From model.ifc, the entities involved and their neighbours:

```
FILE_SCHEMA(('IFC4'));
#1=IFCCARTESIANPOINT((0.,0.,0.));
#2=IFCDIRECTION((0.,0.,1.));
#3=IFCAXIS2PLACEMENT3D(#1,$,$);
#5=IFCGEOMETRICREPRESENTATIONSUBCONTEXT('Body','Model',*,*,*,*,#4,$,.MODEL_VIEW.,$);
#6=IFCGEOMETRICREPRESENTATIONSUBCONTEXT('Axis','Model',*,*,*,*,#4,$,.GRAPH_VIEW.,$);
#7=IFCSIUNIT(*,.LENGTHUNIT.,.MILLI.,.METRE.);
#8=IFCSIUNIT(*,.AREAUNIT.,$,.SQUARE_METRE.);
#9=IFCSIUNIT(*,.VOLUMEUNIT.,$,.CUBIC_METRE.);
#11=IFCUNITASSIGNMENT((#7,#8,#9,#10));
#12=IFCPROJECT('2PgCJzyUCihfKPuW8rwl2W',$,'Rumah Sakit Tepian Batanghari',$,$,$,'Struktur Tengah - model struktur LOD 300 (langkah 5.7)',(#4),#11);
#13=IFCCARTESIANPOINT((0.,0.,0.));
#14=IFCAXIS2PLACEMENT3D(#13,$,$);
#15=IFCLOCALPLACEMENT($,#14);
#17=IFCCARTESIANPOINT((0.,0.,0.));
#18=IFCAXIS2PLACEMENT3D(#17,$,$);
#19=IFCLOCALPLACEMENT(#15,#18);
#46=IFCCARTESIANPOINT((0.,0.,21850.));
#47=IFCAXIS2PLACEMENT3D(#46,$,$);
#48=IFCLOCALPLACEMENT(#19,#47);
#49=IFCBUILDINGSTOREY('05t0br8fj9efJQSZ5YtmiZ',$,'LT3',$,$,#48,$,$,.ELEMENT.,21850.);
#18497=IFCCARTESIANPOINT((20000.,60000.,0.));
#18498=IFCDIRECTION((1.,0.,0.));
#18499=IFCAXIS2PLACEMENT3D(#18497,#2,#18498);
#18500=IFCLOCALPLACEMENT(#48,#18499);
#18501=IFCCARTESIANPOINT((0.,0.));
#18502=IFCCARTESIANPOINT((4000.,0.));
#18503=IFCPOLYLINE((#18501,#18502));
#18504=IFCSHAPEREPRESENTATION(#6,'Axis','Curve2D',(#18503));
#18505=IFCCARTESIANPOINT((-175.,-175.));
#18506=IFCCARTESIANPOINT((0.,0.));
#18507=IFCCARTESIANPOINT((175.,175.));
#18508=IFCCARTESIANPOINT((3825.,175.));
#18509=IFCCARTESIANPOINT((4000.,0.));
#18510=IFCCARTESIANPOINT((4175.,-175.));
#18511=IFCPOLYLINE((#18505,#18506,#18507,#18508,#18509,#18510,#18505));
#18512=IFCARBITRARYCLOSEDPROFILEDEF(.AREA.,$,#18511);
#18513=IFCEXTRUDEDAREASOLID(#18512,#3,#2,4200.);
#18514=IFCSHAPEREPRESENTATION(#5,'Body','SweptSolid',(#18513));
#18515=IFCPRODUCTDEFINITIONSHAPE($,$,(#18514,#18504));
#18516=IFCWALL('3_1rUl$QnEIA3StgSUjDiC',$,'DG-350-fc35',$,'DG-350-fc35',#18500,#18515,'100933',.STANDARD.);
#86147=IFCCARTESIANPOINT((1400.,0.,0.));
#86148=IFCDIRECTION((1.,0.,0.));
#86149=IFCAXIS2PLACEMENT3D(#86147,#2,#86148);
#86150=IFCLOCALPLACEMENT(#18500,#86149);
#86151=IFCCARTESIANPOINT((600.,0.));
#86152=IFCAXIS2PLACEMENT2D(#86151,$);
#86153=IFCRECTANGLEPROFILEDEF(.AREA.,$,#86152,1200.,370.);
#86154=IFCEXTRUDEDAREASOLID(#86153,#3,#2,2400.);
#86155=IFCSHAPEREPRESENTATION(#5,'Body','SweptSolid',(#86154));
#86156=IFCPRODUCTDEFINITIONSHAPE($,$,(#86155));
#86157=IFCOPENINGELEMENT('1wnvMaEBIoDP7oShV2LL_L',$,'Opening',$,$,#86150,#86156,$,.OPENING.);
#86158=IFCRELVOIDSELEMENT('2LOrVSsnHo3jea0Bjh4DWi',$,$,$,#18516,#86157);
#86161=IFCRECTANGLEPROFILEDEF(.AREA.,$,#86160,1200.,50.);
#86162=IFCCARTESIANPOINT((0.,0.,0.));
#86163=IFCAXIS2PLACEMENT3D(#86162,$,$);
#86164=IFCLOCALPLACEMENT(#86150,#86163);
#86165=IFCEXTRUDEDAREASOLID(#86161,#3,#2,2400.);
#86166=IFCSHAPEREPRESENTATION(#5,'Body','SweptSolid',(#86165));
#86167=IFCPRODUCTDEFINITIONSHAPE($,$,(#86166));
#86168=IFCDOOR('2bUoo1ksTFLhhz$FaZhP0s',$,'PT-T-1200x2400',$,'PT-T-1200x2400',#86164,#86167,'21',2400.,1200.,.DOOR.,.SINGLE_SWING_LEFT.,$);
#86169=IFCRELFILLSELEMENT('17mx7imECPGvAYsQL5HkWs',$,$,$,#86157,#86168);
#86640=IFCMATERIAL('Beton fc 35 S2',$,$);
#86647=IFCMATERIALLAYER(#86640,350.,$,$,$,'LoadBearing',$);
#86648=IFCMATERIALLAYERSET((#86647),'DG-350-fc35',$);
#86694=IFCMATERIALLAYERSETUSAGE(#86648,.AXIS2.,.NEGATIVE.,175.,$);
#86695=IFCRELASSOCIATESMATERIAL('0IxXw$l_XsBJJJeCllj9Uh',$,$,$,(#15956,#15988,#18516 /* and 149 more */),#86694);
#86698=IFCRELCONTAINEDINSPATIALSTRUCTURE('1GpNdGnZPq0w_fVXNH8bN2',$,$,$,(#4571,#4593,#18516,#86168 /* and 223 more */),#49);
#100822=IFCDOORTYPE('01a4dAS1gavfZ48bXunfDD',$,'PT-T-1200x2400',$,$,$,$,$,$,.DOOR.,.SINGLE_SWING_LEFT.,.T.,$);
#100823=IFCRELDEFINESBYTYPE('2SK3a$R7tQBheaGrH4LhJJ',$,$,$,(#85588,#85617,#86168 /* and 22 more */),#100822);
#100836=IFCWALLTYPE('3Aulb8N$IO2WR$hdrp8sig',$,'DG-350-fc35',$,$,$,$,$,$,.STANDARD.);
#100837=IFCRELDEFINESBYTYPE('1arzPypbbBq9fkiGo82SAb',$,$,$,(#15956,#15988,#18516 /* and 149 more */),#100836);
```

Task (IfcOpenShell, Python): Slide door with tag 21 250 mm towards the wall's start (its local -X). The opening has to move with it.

```python
import ifcopenshell
import ifcopenshell.api.geometry
import ifcopenshell.util.placement

model = ifcopenshell.open("model.ifc")

door = model.by_guid("2bUoo1ksTFLhhz$FaZhP0s")
opening = door.FillsVoids[0].RelatingOpeningElement
wall = opening.VoidsElements[0].RelatingBuildingElement

wall_matrix = ifcopenshell.util.placement.get_local_placement(wall.ObjectPlacement)
shift = wall_matrix[:3, 0] * -250.0
before = ifcopenshell.util.placement.get_local_placement(door.ObjectPlacement)[:3, 3].copy()

# The door is placed relative to its opening, so it follows when the opening moves.
matrix = ifcopenshell.util.placement.get_local_placement(opening.ObjectPlacement)
matrix[:3, 3] += shift
ifcopenshell.api.geometry.edit_object_placement(
    model, product=opening, matrix=matrix, is_si=False, should_transform_children=True
)

after = ifcopenshell.util.placement.get_local_placement(door.ObjectPlacement)[:3, 3]
print("door moved by", (after - before).round(3) + 0.0)

model.write("model-out.ifc")
```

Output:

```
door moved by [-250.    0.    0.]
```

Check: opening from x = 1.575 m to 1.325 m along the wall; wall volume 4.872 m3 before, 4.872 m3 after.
